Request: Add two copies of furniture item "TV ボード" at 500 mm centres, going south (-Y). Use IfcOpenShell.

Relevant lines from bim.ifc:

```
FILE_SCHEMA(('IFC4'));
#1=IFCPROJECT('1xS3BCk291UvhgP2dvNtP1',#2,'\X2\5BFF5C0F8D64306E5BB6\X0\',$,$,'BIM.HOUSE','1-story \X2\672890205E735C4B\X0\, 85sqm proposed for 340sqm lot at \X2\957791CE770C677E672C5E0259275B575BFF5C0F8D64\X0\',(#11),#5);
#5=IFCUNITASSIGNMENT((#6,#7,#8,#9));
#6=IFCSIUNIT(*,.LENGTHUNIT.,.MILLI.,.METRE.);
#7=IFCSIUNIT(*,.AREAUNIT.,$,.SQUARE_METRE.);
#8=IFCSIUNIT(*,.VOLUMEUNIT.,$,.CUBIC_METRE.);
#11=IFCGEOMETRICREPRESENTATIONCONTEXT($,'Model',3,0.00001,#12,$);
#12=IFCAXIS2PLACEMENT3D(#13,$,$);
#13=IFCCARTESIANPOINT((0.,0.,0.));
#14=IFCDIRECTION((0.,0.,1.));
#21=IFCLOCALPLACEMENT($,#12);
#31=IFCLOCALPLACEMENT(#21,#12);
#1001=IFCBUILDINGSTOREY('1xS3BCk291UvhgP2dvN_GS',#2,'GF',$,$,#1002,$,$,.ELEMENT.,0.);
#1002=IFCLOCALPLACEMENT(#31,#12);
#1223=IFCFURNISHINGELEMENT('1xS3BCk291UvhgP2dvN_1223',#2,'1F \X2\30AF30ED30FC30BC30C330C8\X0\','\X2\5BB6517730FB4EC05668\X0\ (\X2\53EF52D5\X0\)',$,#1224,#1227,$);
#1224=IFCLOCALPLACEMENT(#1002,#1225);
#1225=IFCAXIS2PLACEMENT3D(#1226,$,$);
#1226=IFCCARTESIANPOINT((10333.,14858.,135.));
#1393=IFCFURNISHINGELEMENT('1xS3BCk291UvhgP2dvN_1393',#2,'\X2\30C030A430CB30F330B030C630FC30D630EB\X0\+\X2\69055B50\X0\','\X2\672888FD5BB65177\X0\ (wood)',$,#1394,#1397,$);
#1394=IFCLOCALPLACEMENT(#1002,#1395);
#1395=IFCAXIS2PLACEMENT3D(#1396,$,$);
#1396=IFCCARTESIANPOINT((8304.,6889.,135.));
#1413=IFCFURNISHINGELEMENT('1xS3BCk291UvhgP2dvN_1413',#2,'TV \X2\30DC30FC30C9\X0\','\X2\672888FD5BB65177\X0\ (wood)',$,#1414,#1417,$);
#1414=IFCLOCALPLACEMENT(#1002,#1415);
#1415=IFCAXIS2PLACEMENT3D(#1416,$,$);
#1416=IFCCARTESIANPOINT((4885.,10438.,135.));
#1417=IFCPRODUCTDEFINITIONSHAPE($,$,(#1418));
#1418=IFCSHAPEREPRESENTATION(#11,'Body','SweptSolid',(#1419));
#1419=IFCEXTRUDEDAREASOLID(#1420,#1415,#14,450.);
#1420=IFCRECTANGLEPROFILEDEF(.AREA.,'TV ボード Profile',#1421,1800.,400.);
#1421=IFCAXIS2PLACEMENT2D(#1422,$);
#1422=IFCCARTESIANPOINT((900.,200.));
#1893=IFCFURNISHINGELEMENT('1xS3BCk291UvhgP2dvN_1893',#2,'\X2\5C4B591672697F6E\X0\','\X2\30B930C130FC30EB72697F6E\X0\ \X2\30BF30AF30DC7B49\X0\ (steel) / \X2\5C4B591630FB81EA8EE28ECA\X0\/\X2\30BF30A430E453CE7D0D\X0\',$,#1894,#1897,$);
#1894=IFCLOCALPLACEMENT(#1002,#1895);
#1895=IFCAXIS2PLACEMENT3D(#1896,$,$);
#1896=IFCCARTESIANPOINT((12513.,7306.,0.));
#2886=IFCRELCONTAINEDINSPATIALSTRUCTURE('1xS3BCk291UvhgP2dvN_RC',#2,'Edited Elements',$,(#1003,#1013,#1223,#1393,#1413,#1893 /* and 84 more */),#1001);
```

```python
import numpy as np
import ifcopenshell
import ifcopenshell.api.geometry
import ifcopenshell.api.root
import ifcopenshell.util.element
import ifcopenshell.util.placement

model = ifcopenshell.open("bim.ifc")


def reuse_history(source, copy):
    """copy_class also copies each property set's owner history, people and application; keep the originals."""
    for rel in copy.IsDefinedBy:
        if rel.is_a("IfcRelDefinesByProperties") and (history := rel.RelatingPropertyDefinition.OwnerHistory):
            rel.RelatingPropertyDefinition.OwnerHistory = source.OwnerHistory
            ifcopenshell.util.element.remove_deep2(model, history)


source = model.by_guid("1xS3BCk291UvhgP2dvN_1413")
base = ifcopenshell.util.placement.get_local_placement(source.ObjectPlacement)
step = np.array([0.0, -1.0, 0.0]) * 500.0

for i in range(1, 3):
    copy = ifcopenshell.api.root.copy_class(model, product=source)
    copy.Representation = ifcopenshell.util.element.copy_deep(
        model, source.Representation, exclude=["IfcGeometricRepresentationContext", "IfcRepresentationMap"]
    )
    reuse_history(source, copy)
    matrix = base.copy()
    matrix[:3, 3] += i * step
    print("added at", matrix[:3, 3].round(3) + 0.0)
    ifcopenshell.api.geometry.edit_object_placement(model, product=copy, matrix=matrix, is_si=False)

model.write("bim_updated.ifc")
```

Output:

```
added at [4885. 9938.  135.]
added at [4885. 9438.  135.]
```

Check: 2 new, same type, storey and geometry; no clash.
